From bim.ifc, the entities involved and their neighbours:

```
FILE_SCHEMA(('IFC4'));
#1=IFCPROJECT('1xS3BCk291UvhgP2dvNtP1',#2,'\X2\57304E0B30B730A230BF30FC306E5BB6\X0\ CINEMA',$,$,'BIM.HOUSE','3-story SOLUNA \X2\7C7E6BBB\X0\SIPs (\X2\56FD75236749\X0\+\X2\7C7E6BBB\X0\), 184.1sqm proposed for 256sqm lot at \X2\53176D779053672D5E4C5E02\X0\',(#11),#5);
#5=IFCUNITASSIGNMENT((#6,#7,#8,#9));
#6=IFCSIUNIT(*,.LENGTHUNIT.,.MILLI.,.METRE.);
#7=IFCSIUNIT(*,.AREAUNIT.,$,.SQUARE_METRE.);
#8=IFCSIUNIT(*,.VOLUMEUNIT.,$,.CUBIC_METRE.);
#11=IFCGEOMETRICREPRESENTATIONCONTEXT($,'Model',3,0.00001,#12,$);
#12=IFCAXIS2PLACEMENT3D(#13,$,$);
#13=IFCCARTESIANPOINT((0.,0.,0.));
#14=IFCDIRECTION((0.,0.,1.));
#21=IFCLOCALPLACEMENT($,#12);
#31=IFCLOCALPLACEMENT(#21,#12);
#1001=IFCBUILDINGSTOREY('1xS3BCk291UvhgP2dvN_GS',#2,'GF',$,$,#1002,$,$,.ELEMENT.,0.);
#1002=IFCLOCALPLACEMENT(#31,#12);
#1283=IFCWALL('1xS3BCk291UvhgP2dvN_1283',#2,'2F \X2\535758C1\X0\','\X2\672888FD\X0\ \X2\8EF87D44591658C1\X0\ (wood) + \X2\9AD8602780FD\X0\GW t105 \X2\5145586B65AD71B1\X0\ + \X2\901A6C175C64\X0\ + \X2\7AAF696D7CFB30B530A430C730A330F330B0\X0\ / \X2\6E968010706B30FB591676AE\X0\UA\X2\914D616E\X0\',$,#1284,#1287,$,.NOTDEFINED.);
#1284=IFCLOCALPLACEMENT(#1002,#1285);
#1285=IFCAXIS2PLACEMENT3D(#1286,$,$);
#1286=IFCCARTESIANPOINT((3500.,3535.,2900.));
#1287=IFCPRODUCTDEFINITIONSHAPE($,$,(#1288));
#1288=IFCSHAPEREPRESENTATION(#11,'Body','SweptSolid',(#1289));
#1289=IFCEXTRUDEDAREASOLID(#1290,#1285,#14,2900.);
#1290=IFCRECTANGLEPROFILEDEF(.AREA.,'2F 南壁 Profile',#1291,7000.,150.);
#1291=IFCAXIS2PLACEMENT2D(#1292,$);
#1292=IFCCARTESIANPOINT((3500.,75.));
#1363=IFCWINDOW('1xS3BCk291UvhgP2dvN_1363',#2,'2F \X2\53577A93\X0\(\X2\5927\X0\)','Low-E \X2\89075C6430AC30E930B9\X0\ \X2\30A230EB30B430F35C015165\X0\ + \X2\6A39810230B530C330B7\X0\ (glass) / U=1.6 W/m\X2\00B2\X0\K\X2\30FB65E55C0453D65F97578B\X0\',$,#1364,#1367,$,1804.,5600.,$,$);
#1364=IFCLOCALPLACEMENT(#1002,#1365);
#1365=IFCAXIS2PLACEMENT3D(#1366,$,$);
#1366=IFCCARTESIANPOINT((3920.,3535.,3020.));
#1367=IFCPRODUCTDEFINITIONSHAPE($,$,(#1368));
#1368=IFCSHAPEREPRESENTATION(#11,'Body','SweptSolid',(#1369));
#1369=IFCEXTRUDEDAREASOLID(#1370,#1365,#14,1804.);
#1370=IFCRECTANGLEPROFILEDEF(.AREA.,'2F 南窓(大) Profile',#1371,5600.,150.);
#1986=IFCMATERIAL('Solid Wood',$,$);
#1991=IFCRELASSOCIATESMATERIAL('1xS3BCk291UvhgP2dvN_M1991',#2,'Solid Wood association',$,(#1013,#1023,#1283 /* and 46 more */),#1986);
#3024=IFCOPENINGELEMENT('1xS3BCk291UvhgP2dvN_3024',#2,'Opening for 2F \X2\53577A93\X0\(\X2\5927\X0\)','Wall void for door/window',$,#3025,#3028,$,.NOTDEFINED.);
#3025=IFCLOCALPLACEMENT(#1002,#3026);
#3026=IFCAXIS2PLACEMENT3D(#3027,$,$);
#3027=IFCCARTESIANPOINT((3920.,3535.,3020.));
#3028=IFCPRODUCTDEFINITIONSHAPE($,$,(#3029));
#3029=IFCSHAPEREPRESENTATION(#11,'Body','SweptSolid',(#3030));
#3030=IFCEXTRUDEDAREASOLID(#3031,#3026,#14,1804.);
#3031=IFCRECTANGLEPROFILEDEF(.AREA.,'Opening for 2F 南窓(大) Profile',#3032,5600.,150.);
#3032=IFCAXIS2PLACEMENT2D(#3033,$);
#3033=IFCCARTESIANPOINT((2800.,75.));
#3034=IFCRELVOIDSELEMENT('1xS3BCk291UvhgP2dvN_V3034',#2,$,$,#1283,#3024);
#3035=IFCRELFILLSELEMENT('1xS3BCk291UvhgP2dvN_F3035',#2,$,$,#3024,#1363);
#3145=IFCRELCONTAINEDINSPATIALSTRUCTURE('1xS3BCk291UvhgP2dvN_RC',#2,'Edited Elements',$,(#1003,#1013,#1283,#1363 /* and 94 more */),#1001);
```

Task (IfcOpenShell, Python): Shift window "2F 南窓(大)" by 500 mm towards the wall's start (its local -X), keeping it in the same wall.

```python
import ifcopenshell
import ifcopenshell.api.geometry
import ifcopenshell.util.placement
import ifcopenshell.util.unit

model = ifcopenshell.open("bim.ifc")
unit_scale = ifcopenshell.util.unit.calculate_unit_scale(model)

window = model.by_guid("1xS3BCk291UvhgP2dvN_1363")
opening = window.FillsVoids[0].RelatingOpeningElement
wall = opening.VoidsElements[0].RelatingBuildingElement

wall_matrix = ifcopenshell.util.placement.get_local_placement(wall.ObjectPlacement)
shift = wall_matrix[:3, 0] * -0.5 / unit_scale
before = ifcopenshell.util.placement.get_local_placement(window.ObjectPlacement)[:3, 3].copy()

# The window is not placed relative to its opening, so move both.
for product in (opening, window):
    matrix = ifcopenshell.util.placement.get_local_placement(product.ObjectPlacement)
    matrix[:3, 3] += shift
    ifcopenshell.api.geometry.edit_object_placement(model, product=product, matrix=matrix, is_si=False)

after = ifcopenshell.util.placement.get_local_placement(window.ObjectPlacement)[:3, 3]
print("window moved by", (after - before).round(3) + 0.0)

model.write("bim_rev.ifc")
```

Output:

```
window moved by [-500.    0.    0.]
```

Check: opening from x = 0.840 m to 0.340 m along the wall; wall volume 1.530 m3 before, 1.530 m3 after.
